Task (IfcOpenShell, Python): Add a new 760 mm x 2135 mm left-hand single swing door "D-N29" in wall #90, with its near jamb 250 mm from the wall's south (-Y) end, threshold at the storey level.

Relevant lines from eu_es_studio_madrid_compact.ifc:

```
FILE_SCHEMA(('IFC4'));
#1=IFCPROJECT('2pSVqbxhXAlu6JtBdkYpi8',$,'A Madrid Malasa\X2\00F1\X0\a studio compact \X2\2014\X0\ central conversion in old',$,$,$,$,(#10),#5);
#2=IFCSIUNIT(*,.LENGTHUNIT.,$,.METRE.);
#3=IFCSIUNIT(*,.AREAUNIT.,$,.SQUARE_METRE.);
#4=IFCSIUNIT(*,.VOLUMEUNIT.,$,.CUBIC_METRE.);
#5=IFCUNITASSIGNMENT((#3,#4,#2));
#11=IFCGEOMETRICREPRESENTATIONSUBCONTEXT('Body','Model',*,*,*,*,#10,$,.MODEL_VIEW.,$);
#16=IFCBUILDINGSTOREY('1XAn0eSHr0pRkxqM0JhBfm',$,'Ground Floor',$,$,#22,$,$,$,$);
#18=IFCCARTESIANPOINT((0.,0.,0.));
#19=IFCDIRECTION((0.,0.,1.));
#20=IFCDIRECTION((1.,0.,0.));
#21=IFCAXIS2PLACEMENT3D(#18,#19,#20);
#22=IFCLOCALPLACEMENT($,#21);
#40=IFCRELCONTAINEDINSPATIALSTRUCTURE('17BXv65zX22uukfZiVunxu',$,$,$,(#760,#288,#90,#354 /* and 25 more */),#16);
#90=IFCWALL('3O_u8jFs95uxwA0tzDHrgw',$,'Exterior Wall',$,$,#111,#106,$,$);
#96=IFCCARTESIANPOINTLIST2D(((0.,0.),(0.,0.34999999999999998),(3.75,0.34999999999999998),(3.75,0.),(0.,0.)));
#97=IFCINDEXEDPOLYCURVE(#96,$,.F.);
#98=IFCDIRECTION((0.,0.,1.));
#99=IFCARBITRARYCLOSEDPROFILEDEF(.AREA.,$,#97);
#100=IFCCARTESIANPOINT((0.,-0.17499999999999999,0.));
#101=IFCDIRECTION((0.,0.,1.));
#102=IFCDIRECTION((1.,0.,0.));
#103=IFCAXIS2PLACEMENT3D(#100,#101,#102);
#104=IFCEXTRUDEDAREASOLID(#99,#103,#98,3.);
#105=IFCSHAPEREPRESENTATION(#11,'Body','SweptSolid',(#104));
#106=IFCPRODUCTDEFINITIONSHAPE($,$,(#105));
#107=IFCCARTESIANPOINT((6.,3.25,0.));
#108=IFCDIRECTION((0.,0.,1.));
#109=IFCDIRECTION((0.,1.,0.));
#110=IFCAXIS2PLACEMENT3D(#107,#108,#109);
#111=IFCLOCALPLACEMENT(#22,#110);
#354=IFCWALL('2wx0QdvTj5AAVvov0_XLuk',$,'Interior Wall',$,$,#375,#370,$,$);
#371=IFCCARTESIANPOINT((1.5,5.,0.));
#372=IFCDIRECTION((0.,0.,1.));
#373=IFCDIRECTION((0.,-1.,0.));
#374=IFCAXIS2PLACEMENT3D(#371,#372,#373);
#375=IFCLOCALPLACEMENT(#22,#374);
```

```python
import numpy as np
import ifcopenshell
import ifcopenshell.api.feature
import ifcopenshell.api.geometry
import ifcopenshell.api.root
import ifcopenshell.api.spatial
import ifcopenshell.geom
import ifcopenshell.util.element
import ifcopenshell.util.placement
import ifcopenshell.util.representation
import ifcopenshell.util.shape
import ifcopenshell.util.unit

model = ifcopenshell.open("eu_es_studio_madrid_compact.ifc")
unit_scale = ifcopenshell.util.unit.calculate_unit_scale(model)
settings = ifcopenshell.geom.settings()


def volume(element):
    """Net volume in cubic metres, openings subtracted."""
    shape = ifcopenshell.geom.create_shape(settings, element)
    return ifcopenshell.util.shape.get_volume(shape.geometry)


wall = model.by_id(90)
storey = ifcopenshell.util.element.get_container(wall, ifc_class="IfcBuildingStorey")
context = ifcopenshell.util.representation.get_context(model, "Model", "Body", "MODEL_VIEW")
before = volume(wall)

width, height, from_end, sill = 0.76, 2.135, 0.25, 0.0  # metres

# The wall runs along its own X axis, and the end named is its -X end.
wall_shape = ifcopenshell.geom.create_shape(settings, wall)
x, y, z = ifcopenshell.util.shape.get_vertices(wall_shape.geometry).T
start = x.min() + from_end
face, thickness = float(y.min()), float(y.max() - y.min())
wall_matrix = ifcopenshell.util.placement.get_local_placement(wall.ObjectPlacement)
level = ifcopenshell.util.placement.get_local_placement(storey.ObjectPlacement)[2, 3]


def in_wall(x, y):
    """Placement at x, y metres in the wall's axes, at sill height."""
    matrix = wall_matrix.copy()
    matrix[:, 3] = wall_matrix @ np.array([x / unit_scale, y / unit_scale, 0.0, 1.0])
    matrix[2, 3] = level + sill / unit_scale
    return matrix


# Opening: a box that overshoots both wall faces by 50 mm.
opening = ifcopenshell.api.root.create_entity(model, ifc_class="IfcOpeningElement", predefined_type="OPENING")
box = ifcopenshell.api.geometry.add_wall_representation(
    model, context=context, length=width, height=height, thickness=thickness + 0.1
)
ifcopenshell.api.geometry.assign_representation(model, product=opening, representation=box)
ifcopenshell.api.geometry.edit_object_placement(model, product=opening, matrix=in_wall(start, face - 0.05), is_si=False)
ifcopenshell.api.feature.add_feature(model, feature=opening, element=wall)

door = ifcopenshell.api.root.create_entity(model, ifc_class="IfcDoor", name="D-N29", predefined_type="DOOR")
door.OverallWidth, door.OverallHeight = width / unit_scale, height / unit_scale
door.OperationType = "SINGLE_SWING_LEFT"
body = ifcopenshell.api.geometry.add_door_representation(
    model,
    context=context,
    overall_width=door.OverallWidth,
    overall_height=door.OverallHeight,
    operation_type="SINGLE_SWING_LEFT",
    lining_properties={"LiningDepth": thickness / unit_scale, "ThresholdDepth": thickness / unit_scale},
)
ifcopenshell.api.geometry.assign_representation(model, product=door, representation=body)
ifcopenshell.api.spatial.assign_container(model, products=[door], relating_structure=storey)
ifcopenshell.api.feature.add_filling(model, opening=opening, element=door)

# The lining spans the wall, so the door starts at the wall face.
ifcopenshell.api.geometry.edit_object_placement(model, product=door, matrix=in_wall(start, face), is_si=False)

after = volume(wall)

print(f"wall volume {before:.3f} -> {after:.3f} m3")

model.write("eu_es_studio_madrid_compact_v2.ifc")
```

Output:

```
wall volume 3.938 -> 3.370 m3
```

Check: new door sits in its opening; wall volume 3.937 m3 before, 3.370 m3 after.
